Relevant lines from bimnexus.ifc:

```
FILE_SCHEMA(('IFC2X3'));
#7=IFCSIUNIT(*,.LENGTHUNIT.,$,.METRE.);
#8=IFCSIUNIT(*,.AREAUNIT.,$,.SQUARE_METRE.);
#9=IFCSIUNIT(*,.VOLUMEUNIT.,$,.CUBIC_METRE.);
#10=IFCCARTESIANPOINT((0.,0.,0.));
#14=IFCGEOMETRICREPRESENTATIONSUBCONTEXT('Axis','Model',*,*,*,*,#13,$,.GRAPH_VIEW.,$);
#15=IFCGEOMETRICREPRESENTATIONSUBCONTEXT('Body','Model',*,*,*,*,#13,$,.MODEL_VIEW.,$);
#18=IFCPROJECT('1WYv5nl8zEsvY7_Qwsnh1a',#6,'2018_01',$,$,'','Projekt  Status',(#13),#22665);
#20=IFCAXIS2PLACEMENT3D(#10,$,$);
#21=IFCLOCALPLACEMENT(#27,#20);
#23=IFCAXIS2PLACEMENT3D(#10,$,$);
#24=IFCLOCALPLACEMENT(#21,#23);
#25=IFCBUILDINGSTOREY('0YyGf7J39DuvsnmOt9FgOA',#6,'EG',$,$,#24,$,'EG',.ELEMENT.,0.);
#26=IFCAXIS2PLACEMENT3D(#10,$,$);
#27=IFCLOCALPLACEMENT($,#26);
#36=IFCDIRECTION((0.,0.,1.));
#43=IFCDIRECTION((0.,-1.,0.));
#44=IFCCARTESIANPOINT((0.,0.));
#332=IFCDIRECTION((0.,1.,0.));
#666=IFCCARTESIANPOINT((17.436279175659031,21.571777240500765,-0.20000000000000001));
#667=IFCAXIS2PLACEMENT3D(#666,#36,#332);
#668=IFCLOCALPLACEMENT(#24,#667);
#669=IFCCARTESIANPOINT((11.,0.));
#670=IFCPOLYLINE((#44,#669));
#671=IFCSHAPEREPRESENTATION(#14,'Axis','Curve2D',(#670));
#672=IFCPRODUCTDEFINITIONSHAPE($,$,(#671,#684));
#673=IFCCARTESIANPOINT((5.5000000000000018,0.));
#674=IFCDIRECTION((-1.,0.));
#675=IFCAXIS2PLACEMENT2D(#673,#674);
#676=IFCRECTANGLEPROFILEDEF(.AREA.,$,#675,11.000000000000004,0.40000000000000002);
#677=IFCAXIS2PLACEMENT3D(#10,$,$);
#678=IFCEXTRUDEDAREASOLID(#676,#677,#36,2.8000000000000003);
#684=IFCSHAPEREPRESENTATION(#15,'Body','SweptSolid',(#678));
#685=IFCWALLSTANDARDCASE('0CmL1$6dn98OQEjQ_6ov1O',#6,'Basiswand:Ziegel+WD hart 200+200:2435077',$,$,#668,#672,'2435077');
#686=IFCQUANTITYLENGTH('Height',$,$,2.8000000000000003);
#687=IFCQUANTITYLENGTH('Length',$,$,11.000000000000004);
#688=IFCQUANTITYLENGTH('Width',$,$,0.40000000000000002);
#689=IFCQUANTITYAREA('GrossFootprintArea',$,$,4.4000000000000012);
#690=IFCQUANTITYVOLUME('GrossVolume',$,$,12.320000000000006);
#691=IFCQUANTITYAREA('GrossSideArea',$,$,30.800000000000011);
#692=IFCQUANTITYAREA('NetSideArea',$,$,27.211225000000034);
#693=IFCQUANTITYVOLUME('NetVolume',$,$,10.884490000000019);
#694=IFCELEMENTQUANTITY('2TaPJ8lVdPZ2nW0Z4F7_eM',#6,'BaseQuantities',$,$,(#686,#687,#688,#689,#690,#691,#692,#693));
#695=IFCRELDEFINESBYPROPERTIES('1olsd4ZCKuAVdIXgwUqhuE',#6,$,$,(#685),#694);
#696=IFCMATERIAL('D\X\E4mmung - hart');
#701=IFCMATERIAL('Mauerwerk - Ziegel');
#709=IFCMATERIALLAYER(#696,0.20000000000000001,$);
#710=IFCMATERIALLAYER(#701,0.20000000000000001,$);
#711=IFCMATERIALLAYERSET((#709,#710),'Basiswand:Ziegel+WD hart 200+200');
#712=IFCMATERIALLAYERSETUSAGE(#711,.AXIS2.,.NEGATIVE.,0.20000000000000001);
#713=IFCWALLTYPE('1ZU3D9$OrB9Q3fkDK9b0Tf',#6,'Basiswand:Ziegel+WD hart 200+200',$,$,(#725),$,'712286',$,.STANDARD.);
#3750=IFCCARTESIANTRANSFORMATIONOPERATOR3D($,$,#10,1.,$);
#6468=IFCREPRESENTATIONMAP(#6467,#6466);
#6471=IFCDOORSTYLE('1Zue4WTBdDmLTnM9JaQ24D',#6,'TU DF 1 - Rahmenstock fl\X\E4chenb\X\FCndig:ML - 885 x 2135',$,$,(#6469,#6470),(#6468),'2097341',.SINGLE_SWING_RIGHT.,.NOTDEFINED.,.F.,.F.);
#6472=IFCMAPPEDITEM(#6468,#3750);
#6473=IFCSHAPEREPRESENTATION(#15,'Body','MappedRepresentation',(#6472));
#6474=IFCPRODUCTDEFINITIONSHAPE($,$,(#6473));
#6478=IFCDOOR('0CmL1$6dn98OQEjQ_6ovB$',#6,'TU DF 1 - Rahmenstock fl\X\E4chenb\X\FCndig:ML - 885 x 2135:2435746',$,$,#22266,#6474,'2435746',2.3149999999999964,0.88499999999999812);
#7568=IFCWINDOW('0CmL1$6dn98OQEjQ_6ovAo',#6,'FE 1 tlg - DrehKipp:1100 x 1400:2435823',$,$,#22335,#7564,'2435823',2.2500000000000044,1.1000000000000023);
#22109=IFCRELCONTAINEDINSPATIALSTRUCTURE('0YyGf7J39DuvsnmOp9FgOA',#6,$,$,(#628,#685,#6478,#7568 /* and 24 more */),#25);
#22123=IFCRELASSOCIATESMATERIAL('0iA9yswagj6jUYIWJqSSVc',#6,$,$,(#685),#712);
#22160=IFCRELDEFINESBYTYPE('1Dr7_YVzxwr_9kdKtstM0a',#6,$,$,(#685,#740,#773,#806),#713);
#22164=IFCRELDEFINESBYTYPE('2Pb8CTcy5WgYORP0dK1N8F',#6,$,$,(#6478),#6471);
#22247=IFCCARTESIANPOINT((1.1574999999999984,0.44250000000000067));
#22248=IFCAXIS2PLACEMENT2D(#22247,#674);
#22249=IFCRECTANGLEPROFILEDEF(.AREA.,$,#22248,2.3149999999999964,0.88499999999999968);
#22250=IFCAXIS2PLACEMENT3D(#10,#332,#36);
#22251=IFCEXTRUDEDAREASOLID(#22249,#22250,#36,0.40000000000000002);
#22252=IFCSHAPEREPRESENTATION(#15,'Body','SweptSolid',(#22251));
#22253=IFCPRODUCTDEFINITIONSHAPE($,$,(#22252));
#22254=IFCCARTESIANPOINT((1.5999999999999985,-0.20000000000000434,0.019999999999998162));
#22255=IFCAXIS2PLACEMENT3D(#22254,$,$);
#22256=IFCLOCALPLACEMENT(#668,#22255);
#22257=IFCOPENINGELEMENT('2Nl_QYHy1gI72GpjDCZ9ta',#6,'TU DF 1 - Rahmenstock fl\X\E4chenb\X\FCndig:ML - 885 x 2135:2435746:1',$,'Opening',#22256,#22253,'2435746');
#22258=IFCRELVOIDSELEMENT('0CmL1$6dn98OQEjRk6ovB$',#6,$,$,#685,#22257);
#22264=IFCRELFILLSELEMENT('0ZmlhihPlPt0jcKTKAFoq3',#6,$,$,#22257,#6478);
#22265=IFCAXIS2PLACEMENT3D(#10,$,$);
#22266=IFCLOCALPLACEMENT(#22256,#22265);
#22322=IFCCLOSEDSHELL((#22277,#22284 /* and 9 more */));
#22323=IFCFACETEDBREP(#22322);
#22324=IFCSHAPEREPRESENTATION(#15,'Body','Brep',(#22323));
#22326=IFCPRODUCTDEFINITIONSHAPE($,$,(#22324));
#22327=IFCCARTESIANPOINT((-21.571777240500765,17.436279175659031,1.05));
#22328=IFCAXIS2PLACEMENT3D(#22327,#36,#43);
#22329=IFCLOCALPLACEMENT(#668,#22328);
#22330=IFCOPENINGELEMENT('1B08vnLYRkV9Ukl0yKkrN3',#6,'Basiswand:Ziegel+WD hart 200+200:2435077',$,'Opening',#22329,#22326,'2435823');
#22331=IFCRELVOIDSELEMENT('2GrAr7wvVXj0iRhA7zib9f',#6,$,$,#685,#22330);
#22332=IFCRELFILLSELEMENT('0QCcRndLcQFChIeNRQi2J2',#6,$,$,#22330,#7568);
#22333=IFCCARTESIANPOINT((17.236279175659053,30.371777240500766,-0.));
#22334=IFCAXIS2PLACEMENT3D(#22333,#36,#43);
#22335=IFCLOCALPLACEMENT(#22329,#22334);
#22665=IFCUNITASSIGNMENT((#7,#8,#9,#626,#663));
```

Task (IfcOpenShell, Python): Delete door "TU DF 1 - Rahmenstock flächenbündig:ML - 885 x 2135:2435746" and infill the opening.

```python
import ifcopenshell
import ifcopenshell.api.feature
import ifcopenshell.api.pset
import ifcopenshell.api.root
import ifcopenshell.geom
import ifcopenshell.util.element
import ifcopenshell.util.shape
import ifcopenshell.util.unit

model = ifcopenshell.open("bimnexus.ifc")
area_scale = ifcopenshell.util.unit.calculate_unit_scale(model, "AREAUNIT")
volume_scale = ifcopenshell.util.unit.calculate_unit_scale(model, "VOLUMEUNIT")
settings = ifcopenshell.geom.settings()


def volume(element):
    """Net volume in cubic metres, openings subtracted."""
    shape = ifcopenshell.geom.create_shape(settings, element)
    return ifcopenshell.util.shape.get_volume(shape.geometry)


door = model.by_id(6478)
opening = door.FillsVoids[0].RelatingOpeningElement
wall = opening.VoidsElements[0].RelatingBuildingElement
before = volume(wall)

ifcopenshell.api.root.remove_product(model, product=door)
ifcopenshell.api.feature.remove_feature(model, feature=opening)

after = volume(wall)
thickness = 0.4  # wall thickness in metres

# Update the wall's stored quantities.
qto = model.by_id(ifcopenshell.util.element.get_pset(wall, "BaseQuantities", should_inherit=False)["id"])
ifcopenshell.api.pset.edit_qto(model, qto=qto, properties={
    "NetSideArea": after / thickness / area_scale,
    "NetVolume": after / volume_scale,
})

print(f"wall volume {before:.3f} -> {after:.3f} m3")

model.write("bimnexus_updated.ifc")
```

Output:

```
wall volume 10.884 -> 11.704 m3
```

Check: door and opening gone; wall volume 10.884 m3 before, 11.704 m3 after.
